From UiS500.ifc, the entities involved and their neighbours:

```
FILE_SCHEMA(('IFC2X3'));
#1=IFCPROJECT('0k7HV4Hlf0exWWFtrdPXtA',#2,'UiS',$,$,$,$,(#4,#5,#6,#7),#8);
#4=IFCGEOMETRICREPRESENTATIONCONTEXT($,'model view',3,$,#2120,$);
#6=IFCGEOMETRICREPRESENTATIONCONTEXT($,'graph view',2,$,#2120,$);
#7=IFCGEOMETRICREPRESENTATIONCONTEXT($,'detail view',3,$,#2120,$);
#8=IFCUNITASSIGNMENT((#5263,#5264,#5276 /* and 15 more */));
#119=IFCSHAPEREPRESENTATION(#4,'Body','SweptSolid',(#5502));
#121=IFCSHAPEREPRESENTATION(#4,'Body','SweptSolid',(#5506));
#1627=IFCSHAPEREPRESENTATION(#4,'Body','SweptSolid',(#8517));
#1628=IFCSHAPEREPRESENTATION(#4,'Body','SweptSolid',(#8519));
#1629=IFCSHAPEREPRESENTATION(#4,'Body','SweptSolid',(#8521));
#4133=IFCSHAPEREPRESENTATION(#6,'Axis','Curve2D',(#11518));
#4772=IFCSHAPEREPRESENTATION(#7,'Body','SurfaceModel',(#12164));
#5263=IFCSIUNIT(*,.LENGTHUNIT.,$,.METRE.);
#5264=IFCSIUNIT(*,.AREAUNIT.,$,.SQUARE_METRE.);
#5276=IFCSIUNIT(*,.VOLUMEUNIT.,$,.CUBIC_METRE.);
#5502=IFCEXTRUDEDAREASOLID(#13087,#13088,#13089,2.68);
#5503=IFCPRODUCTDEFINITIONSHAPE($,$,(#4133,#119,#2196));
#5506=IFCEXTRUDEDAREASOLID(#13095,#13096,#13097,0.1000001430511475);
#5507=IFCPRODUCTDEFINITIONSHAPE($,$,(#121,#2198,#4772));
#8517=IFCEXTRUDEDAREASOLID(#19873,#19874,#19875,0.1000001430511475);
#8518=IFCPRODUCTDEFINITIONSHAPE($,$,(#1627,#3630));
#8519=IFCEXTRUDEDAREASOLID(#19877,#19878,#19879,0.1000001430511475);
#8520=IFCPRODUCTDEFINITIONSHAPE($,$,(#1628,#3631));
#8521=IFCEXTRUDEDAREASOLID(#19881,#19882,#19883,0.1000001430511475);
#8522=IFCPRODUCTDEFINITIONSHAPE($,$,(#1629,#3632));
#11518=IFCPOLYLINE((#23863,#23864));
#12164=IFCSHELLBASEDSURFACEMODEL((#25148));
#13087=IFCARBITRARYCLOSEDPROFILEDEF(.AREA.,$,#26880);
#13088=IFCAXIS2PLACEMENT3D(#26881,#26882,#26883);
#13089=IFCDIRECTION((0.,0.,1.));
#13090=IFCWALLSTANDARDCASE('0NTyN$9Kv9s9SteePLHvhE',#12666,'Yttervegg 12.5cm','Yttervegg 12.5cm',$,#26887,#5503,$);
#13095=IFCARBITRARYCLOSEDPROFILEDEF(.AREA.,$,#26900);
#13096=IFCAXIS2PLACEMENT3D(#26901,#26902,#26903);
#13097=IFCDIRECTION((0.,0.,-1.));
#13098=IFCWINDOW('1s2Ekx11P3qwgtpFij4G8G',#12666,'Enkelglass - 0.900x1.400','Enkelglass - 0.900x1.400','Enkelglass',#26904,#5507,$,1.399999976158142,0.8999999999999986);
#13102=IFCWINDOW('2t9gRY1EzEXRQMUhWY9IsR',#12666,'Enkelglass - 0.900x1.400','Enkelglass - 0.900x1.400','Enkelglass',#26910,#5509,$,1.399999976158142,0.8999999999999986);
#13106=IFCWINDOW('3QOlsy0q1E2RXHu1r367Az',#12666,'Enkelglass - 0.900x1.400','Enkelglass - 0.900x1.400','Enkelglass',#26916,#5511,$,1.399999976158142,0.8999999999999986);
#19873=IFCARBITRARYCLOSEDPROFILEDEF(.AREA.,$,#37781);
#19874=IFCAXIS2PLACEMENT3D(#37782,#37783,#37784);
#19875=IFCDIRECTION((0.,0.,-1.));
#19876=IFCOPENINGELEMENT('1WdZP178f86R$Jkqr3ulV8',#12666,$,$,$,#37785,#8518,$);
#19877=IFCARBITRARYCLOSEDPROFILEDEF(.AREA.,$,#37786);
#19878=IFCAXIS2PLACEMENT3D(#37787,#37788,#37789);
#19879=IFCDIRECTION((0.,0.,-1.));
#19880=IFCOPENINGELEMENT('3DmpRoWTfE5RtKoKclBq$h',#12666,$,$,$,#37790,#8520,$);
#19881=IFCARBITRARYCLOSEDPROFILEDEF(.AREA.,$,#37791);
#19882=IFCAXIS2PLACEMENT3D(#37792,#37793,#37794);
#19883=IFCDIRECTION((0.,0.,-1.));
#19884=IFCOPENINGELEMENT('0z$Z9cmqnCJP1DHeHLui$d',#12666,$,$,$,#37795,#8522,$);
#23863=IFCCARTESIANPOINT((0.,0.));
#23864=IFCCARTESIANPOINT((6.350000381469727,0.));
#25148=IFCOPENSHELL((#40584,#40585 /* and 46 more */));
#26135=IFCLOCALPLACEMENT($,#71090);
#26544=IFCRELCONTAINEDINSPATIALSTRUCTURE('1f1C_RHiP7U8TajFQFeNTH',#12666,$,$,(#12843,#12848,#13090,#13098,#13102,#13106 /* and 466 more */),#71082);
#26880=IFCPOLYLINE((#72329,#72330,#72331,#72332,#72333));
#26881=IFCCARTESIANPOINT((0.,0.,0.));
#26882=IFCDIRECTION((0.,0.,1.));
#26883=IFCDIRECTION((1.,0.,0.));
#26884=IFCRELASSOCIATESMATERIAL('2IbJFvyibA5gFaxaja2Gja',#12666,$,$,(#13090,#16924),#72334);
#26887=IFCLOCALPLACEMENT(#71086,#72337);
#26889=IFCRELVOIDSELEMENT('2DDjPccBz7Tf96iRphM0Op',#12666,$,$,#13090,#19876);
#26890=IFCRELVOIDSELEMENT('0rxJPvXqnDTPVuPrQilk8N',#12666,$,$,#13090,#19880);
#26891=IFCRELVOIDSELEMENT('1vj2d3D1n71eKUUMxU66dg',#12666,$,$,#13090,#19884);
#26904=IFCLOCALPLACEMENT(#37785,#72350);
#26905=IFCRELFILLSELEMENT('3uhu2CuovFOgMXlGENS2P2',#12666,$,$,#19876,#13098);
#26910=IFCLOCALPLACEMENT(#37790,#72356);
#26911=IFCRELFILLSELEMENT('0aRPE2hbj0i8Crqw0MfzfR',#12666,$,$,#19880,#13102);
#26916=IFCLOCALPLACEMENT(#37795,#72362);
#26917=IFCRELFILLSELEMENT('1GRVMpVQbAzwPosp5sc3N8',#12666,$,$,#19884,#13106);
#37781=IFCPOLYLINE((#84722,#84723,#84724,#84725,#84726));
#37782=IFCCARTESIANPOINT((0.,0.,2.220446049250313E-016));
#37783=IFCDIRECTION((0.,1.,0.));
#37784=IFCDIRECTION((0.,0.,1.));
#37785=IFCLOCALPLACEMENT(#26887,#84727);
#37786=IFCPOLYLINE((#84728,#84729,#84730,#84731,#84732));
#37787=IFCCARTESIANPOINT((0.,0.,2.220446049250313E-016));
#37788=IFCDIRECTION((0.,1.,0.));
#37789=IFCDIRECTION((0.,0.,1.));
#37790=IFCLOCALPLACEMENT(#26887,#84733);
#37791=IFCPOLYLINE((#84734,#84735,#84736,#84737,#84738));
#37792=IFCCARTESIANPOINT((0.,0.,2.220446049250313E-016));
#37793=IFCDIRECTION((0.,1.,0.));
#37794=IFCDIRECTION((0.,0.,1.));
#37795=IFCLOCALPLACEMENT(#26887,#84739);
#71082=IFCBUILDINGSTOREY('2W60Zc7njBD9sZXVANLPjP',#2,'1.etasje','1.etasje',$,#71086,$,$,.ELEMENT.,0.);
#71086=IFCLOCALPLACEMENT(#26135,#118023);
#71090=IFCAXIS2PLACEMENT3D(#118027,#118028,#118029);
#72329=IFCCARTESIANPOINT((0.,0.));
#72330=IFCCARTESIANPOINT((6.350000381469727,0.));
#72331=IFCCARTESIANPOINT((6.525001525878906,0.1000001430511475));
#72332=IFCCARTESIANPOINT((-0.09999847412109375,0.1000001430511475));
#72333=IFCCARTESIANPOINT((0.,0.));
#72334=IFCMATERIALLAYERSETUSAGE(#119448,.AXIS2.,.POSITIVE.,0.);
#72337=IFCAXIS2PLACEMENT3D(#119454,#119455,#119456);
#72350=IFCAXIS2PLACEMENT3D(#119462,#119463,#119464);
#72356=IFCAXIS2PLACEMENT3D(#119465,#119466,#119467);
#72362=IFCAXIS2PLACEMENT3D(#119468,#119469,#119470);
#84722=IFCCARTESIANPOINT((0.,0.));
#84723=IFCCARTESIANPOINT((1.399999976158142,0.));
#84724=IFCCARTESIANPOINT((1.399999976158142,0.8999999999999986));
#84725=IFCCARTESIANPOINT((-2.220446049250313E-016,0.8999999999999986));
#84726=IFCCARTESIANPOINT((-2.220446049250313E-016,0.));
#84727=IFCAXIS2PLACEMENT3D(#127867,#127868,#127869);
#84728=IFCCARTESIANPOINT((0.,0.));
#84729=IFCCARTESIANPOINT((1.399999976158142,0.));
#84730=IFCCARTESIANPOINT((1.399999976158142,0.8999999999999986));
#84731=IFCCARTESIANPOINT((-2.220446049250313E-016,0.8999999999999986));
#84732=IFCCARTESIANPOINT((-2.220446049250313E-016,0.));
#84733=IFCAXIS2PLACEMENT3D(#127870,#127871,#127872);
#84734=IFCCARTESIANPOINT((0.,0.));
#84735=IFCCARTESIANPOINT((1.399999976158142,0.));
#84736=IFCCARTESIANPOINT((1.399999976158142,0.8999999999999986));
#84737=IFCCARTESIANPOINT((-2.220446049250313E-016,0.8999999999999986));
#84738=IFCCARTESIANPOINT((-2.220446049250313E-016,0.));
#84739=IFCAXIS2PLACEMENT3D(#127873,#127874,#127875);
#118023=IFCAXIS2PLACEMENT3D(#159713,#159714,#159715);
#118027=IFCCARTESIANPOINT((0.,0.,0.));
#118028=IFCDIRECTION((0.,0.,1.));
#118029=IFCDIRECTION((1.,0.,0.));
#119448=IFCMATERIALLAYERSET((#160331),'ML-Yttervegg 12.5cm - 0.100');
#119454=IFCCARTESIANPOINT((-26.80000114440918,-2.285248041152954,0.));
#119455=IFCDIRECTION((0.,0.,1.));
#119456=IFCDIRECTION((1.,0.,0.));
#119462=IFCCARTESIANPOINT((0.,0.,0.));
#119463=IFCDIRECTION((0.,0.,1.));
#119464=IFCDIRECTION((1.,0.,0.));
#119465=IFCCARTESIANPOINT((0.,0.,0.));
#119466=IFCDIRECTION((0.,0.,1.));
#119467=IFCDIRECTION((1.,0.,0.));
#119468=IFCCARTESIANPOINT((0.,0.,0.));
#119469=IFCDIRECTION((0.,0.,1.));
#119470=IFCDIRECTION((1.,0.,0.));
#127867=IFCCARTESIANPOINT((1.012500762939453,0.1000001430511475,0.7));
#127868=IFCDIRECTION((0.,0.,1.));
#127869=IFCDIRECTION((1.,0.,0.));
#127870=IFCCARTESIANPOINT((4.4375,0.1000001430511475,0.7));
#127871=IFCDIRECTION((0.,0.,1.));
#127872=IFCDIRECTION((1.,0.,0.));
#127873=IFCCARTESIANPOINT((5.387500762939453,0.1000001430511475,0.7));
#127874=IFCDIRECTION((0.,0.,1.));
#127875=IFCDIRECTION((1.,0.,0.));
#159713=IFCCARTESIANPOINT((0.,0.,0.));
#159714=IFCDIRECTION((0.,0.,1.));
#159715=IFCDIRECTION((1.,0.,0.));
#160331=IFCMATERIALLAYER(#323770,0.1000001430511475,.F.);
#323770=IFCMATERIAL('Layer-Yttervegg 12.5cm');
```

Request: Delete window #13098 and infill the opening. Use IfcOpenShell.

```python
import ifcopenshell
import ifcopenshell.api.feature
import ifcopenshell.api.root
import ifcopenshell.geom
import ifcopenshell.util.shape

model = ifcopenshell.open("UiS500.ifc")
settings = ifcopenshell.geom.settings()


def volume(element):
    """Net volume in cubic metres, openings subtracted."""
    shape = ifcopenshell.geom.create_shape(settings, element)
    return ifcopenshell.util.shape.get_volume(shape.geometry)


window = model.by_guid("1s2Ekx11P3qwgtpFij4G8G")
opening = window.FillsVoids[0].RelatingOpeningElement
wall = opening.VoidsElements[0].RelatingBuildingElement
before = volume(wall)

ifcopenshell.api.root.remove_product(model, product=window)
ifcopenshell.api.feature.remove_feature(model, feature=opening)

after = volume(wall)

print(f"wall volume {before:.3f} -> {after:.3f} m3")

model.write("UiS500_updated.ifc")
```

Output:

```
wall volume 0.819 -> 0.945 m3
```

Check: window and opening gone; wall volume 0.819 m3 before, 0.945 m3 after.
